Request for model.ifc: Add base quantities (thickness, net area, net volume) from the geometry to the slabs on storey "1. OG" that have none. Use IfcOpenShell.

First a look at what the model holds.

```python
import ifcopenshell
import ifcopenshell.util.element
import ifcopenshell.util.unit

model = ifcopenshell.open("model.ifc")
print(model.schema)
for unit_type in ("LENGTHUNIT", "AREAUNIT", "VOLUMEUNIT"):
    print(unit_type, ifcopenshell.util.unit.calculate_unit_scale(model, unit_type))
storey = next(s for s in model.by_type("IfcBuildingStorey") if s.Name == "1. OG")
slabs = [e for e in ifcopenshell.util.element.get_decomposition(storey) if e.is_a("IfcSlab")]
for e in sorted(slabs, key=lambda e: e.id()):
    print(e.id(), e.is_a(), e.Name, list(ifcopenshell.util.element.get_psets(e, qtos_only=True)), sep=" | ")
```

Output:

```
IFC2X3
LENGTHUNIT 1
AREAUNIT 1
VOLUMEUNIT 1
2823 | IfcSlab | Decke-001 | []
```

```python
import ifcopenshell
import ifcopenshell.api.pset
import ifcopenshell.geom
import ifcopenshell.util.element
import ifcopenshell.util.shape
import ifcopenshell.util.unit

model = ifcopenshell.open("model.ifc")
unit_scale = ifcopenshell.util.unit.calculate_unit_scale(model)
area_scale = ifcopenshell.util.unit.calculate_unit_scale(model, "AREAUNIT")
volume_scale = ifcopenshell.util.unit.calculate_unit_scale(model, "VOLUMEUNIT")
settings = ifcopenshell.geom.settings()

storey = next(s for s in model.by_type("IfcBuildingStorey") if s.Name == "1. OG")
slabs = [e for e in ifcopenshell.util.element.get_decomposition(storey) if e.is_a("IfcSlab")]

for e in sorted(slabs, key=lambda e: e.id()):
    if ifcopenshell.util.element.get_psets(e, qtos_only=True, should_inherit=False):
        continue
    # Geometry comes back in metres, in the element's own axes.
    shape = ifcopenshell.geom.create_shape(settings, e)
    values = {
        "Width": ifcopenshell.util.shape.get_z(shape.geometry) / unit_scale,
        "NetArea": ifcopenshell.util.shape.get_footprint_area(shape.geometry) / area_scale,
        "NetVolume": ifcopenshell.util.shape.get_volume(shape.geometry) / volume_scale,
    }
    qto = ifcopenshell.api.pset.add_qto(model, product=e, name="BaseQuantities")
    ifcopenshell.api.pset.edit_qto(model, qto=qto, properties=values)
    print(e.id(), {k: round(v, 3) for k, v in values.items()})

model.write("model_rev.ifc")
```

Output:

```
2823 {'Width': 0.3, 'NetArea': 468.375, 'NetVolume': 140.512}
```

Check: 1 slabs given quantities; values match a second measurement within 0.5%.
